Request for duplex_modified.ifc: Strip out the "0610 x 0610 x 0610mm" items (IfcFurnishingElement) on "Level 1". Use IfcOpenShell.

First a look at what the model holds.

```python
import ifcopenshell
import ifcopenshell.util.element

model = ifcopenshell.open("duplex_modified.ifc")
print(model.schema)
storey = next(s for s in model.by_type("IfcBuildingStorey") if s.Name == "Level 1")
furniture = [e for e in ifcopenshell.util.element.get_decomposition(storey) if e.is_a("IfcFurnishingElement")]
seen = {}
for e in furniture:
    element_type = ifcopenshell.util.element.get_type(e)
    name = element_type.Name if element_type not in (None, e) else None
    seen[name] = seen.get(name, 0) + 1
for name, count in sorted(seen.items(), key=str):
    print(count, "x", name)
```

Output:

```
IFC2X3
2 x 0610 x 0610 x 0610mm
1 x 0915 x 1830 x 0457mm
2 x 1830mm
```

```python
import ifcopenshell
import ifcopenshell.api.root
import ifcopenshell.util.element

model = ifcopenshell.open("duplex_modified.ifc")

storey = next(s for s in model.by_type("IfcBuildingStorey") if s.Name == "Level 1")
furniture = [e for e in ifcopenshell.util.element.get_decomposition(storey) if e.is_a("IfcFurnishingElement")]
targets = [e for e in furniture if (t := ifcopenshell.util.element.get_type(e)) not in (None, e) and t.Name == "0610 x 0610 x 0610mm"]

for e in targets:
    ifcopenshell.api.root.remove_product(model, product=e)
print(len(targets), "removed")

model.write("duplex_modified-out.ifc")
```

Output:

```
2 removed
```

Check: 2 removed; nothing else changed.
